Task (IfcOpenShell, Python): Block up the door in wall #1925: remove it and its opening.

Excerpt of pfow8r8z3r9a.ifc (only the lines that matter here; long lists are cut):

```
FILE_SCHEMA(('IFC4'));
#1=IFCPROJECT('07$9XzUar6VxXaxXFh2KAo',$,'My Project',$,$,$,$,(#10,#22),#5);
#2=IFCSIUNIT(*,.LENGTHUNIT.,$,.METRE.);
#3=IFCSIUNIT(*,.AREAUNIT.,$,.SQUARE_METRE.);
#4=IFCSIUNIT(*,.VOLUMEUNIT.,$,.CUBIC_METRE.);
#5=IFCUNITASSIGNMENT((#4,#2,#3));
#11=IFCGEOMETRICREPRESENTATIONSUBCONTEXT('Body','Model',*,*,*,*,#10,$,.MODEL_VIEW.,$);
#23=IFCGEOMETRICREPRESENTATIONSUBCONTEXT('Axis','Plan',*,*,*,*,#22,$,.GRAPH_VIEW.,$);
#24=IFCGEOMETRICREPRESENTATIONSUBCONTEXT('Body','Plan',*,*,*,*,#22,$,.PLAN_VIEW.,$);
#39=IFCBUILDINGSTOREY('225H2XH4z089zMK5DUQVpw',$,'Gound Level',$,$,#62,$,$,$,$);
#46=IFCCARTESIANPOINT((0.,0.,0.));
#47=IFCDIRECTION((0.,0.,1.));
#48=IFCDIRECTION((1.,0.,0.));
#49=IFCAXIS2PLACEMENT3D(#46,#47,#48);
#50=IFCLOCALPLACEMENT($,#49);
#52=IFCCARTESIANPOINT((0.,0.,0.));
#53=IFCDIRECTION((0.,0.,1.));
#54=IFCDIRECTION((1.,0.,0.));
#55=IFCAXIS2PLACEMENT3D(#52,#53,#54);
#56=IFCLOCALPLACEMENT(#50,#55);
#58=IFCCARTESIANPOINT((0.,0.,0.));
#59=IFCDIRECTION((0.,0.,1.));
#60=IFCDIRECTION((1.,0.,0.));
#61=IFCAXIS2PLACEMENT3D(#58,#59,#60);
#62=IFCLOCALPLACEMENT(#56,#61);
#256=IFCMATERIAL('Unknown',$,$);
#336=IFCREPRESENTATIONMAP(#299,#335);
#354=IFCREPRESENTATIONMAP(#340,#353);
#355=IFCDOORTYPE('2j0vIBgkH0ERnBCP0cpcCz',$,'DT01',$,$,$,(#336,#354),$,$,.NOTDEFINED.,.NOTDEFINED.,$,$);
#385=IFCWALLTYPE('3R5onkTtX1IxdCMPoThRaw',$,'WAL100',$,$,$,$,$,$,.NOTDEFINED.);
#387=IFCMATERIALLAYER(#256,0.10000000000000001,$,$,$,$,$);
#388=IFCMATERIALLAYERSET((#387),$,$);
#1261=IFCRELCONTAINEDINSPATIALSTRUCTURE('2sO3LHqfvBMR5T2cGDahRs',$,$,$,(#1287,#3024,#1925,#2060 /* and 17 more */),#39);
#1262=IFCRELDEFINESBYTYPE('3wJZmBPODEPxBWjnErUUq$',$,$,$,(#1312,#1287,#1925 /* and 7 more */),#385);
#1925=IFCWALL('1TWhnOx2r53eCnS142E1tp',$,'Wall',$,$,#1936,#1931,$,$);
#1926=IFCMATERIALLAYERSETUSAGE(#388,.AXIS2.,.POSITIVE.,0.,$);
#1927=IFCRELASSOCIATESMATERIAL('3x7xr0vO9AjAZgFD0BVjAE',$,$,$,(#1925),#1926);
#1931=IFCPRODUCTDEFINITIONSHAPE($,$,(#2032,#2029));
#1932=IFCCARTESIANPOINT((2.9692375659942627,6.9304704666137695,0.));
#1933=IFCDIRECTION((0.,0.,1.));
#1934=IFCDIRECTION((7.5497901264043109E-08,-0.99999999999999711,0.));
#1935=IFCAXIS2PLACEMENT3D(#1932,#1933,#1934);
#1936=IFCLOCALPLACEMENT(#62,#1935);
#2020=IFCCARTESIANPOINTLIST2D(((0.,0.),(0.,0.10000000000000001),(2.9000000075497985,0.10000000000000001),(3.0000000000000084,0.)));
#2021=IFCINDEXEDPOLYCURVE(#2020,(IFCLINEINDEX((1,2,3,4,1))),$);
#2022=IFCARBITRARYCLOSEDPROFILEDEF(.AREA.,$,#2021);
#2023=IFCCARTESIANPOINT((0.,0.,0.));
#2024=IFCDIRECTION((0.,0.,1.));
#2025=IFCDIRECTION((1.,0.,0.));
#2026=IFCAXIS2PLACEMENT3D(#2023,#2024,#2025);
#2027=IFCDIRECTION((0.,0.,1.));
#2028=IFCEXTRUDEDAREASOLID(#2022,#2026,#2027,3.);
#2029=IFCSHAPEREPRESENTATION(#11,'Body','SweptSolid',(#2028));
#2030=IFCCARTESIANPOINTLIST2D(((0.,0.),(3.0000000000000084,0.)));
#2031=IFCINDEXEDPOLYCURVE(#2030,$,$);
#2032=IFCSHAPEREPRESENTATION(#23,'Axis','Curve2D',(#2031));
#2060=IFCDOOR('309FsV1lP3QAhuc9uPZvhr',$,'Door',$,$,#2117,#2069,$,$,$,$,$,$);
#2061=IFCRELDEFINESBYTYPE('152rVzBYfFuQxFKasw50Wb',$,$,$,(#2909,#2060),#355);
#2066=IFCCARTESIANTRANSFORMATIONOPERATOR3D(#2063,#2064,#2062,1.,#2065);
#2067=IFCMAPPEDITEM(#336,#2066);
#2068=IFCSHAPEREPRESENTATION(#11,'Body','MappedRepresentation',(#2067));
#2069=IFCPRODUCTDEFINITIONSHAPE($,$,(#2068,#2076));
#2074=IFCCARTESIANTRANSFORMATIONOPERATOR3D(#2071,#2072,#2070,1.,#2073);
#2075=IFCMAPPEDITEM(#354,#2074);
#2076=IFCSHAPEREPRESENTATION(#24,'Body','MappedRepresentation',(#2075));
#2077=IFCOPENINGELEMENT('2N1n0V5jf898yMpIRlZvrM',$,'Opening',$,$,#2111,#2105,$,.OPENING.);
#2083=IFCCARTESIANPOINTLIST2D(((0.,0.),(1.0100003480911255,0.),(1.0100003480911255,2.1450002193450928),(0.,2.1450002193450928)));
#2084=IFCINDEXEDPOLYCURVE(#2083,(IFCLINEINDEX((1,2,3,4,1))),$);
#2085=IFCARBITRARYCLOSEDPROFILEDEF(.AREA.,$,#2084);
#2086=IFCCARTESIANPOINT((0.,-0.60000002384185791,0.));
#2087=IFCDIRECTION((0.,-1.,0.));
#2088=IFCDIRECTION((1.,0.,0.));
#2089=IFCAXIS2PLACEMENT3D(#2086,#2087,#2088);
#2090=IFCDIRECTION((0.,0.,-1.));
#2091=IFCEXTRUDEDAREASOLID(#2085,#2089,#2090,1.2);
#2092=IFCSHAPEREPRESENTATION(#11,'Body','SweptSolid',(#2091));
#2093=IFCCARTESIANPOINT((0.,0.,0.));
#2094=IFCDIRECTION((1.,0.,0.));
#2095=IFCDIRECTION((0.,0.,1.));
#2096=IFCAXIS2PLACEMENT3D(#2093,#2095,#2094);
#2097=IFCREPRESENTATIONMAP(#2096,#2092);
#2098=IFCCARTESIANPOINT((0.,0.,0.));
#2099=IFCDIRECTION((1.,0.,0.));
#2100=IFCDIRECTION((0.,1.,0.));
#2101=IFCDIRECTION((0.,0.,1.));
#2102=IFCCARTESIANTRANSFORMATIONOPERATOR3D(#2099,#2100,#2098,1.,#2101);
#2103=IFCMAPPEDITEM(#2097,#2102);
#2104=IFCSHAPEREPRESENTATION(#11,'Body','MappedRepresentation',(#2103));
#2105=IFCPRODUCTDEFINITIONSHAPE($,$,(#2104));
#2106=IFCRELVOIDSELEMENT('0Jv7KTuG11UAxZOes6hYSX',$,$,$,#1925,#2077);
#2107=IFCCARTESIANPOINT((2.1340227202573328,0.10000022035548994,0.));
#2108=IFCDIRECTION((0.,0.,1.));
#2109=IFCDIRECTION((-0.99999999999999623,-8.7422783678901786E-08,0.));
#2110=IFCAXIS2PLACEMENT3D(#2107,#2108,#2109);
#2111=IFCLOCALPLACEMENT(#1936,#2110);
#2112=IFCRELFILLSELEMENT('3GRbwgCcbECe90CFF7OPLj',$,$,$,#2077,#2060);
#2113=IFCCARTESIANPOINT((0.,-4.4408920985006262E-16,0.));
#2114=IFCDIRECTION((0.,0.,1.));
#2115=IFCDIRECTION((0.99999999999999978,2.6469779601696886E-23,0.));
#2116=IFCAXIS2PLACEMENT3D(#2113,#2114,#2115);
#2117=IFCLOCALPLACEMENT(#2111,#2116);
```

```python
import ifcopenshell
import ifcopenshell.api.feature
import ifcopenshell.api.root
import ifcopenshell.geom
import ifcopenshell.util.shape

model = ifcopenshell.open("pfow8r8z3r9a.ifc")
settings = ifcopenshell.geom.settings()


def volume(element):
    """Net volume in cubic metres, openings subtracted."""
    shape = ifcopenshell.geom.create_shape(settings, element)
    return ifcopenshell.util.shape.get_volume(shape.geometry)


door = model.by_guid("309FsV1lP3QAhuc9uPZvhr")
opening = door.FillsVoids[0].RelatingOpeningElement
wall = opening.VoidsElements[0].RelatingBuildingElement
before = volume(wall)

ifcopenshell.api.root.remove_product(model, product=door)
ifcopenshell.api.feature.remove_feature(model, feature=opening)

after = volume(wall)

print(f"wall volume {before:.3f} -> {after:.3f} m3")

model.write("pfow8r8z3r9a_rev.ifc")
```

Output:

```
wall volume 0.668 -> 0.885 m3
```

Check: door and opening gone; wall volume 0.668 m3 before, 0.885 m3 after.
